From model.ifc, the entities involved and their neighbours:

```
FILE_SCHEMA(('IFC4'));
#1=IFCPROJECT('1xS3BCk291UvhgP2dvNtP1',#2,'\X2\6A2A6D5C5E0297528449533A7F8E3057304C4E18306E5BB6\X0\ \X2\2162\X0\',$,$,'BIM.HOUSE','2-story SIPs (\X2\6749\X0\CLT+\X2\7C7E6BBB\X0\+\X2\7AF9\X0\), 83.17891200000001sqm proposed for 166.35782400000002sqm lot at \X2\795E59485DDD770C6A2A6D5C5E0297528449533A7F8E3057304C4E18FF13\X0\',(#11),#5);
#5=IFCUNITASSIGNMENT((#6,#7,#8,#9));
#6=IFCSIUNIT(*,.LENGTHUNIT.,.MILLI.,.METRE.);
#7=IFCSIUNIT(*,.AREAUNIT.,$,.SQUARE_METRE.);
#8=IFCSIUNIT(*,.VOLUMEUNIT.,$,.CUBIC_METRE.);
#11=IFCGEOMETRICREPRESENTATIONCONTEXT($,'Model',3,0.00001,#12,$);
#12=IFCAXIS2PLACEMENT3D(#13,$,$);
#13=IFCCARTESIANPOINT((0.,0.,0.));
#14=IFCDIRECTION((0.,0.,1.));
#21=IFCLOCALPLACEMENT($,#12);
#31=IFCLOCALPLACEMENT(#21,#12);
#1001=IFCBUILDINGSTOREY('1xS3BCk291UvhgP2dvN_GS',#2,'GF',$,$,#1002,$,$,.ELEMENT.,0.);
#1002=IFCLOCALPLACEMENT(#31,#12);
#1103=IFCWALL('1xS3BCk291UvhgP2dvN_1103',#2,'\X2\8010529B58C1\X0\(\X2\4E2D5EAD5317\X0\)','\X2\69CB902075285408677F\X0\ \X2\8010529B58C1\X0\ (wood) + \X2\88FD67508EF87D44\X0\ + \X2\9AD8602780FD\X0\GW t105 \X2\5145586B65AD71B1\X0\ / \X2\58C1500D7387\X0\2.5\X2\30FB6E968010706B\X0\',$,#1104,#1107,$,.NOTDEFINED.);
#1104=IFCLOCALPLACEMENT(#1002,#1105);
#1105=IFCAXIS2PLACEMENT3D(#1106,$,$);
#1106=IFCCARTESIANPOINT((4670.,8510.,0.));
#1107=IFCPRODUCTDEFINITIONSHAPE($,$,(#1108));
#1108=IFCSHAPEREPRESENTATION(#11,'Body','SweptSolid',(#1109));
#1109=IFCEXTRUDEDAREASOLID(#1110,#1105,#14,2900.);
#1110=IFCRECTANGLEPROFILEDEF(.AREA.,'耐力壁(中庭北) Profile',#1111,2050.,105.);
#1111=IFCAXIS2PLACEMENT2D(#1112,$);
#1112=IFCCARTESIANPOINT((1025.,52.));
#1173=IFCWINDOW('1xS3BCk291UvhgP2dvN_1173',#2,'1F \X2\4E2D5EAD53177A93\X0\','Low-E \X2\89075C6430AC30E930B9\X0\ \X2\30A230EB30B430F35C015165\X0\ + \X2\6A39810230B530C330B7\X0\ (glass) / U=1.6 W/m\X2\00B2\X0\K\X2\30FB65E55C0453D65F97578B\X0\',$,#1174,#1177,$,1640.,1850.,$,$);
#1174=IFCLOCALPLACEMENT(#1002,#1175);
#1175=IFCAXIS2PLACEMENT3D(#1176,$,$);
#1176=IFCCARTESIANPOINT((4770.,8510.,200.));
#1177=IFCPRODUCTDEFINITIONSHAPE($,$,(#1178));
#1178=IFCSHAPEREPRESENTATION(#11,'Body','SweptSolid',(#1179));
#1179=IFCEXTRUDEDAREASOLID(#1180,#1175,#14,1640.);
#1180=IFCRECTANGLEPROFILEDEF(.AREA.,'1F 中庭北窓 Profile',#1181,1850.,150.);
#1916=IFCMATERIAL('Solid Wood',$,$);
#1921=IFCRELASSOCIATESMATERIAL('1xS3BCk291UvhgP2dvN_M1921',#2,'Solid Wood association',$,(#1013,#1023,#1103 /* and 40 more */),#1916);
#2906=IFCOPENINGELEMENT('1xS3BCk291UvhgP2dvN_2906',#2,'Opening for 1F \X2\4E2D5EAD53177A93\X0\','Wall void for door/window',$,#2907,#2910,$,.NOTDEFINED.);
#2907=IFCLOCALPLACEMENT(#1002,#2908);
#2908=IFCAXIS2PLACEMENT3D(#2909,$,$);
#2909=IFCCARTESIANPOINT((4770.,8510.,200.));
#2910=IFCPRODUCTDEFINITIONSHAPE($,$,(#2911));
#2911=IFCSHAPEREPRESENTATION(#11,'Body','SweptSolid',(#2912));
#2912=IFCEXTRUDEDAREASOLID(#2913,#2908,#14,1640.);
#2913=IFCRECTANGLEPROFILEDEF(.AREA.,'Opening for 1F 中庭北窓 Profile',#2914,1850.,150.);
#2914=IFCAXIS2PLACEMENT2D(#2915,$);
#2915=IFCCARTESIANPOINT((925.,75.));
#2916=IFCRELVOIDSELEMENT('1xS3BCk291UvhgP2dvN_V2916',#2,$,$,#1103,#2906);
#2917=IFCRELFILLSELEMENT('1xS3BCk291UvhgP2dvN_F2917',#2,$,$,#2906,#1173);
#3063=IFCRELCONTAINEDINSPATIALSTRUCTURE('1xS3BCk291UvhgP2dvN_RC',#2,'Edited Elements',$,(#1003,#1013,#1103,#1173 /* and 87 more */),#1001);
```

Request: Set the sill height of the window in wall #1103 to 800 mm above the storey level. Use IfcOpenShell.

```python
import numpy as np
import ifcopenshell
import ifcopenshell.api.geometry
import ifcopenshell.geom
import ifcopenshell.util.element
import ifcopenshell.util.placement
import ifcopenshell.util.shape
import ifcopenshell.util.unit

model = ifcopenshell.open("model.ifc")
unit_scale = ifcopenshell.util.unit.calculate_unit_scale(model)

window = model.by_id(1173)
opening = window.FillsVoids[0].RelatingOpeningElement
storey = ifcopenshell.util.element.get_container(window, ifc_class="IfcBuildingStorey")
level = ifcopenshell.util.placement.get_local_placement(storey.ObjectPlacement)[2, 3]

# The opening's origin need not be at the sill, so measure its lowest point.
shape = ifcopenshell.geom.create_shape(ifcopenshell.geom.settings(), opening)
bottom = ifcopenshell.util.shape.get_shape_bottom_elevation(shape, shape.geometry) / unit_scale
dz = level + 800.0 - bottom

shift = np.array([0.0, 0.0, dz])
# The window is not placed relative to its opening, so move both.
for product in (opening, window):
    matrix = ifcopenshell.util.placement.get_local_placement(product.ObjectPlacement)
    matrix[:3, 3] += shift
    ifcopenshell.api.geometry.edit_object_placement(model, product=product, matrix=matrix, is_si=False)

print(f"moved by {dz * unit_scale:+.3f} m")

model.write("model_v2.ifc")
```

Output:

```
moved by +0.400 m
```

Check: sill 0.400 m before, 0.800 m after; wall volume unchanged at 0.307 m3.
